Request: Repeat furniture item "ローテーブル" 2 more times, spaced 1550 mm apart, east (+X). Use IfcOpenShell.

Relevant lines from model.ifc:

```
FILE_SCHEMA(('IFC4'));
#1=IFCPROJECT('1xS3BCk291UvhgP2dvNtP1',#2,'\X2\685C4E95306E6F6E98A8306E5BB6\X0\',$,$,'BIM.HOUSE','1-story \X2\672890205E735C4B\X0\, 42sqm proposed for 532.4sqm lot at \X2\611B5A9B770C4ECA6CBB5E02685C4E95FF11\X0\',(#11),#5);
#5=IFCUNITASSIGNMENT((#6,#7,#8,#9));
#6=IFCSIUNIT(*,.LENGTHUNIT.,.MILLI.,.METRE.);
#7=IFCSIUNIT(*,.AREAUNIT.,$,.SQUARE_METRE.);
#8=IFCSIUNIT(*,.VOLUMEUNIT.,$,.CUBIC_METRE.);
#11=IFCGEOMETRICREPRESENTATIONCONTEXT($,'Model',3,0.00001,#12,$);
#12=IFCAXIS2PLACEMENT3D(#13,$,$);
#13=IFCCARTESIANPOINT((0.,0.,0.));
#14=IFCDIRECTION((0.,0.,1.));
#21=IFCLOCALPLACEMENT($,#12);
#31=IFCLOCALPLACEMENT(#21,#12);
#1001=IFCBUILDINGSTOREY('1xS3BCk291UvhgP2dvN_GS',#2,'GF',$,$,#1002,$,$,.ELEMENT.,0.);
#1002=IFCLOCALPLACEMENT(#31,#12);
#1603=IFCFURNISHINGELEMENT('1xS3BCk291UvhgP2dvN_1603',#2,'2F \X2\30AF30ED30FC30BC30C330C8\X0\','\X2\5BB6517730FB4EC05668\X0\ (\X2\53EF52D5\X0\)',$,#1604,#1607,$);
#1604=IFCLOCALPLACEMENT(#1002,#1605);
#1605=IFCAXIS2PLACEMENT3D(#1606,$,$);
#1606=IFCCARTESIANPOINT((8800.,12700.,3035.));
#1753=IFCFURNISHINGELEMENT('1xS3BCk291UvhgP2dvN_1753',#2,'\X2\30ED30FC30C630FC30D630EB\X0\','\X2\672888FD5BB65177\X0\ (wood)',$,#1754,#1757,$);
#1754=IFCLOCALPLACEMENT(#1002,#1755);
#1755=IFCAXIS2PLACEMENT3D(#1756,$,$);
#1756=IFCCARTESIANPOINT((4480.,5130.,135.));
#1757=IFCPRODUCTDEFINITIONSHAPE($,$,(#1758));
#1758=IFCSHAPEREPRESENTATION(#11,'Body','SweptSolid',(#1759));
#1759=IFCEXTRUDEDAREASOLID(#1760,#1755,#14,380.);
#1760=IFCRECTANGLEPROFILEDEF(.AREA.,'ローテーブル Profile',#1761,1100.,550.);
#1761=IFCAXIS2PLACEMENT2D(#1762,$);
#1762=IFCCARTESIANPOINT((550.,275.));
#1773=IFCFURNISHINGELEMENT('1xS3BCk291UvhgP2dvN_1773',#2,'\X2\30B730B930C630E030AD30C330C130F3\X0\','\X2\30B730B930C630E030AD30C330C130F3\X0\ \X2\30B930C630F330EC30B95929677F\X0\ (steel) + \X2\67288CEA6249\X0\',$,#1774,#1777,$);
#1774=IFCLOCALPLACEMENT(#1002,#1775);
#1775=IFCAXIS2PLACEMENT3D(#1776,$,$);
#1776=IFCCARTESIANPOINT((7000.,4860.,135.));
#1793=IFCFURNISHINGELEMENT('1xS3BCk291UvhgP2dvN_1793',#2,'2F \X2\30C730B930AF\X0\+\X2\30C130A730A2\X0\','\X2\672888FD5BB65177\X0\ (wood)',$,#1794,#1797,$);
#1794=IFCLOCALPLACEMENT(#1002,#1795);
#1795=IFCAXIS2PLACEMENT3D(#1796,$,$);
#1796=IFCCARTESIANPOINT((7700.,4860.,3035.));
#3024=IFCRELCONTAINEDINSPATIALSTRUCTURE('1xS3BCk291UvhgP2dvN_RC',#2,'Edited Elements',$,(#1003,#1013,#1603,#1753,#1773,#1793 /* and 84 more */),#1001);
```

```python
import numpy as np
import ifcopenshell
import ifcopenshell.api.geometry
import ifcopenshell.api.root
import ifcopenshell.util.element
import ifcopenshell.util.placement

model = ifcopenshell.open("model.ifc")


def reuse_history(source, copy):
    """copy_class also copies each property set's owner history, people and application; keep the originals."""
    for rel in copy.IsDefinedBy:
        if rel.is_a("IfcRelDefinesByProperties") and (history := rel.RelatingPropertyDefinition.OwnerHistory):
            rel.RelatingPropertyDefinition.OwnerHistory = source.OwnerHistory
            ifcopenshell.util.element.remove_deep2(model, history)


source = model.by_guid("1xS3BCk291UvhgP2dvN_1753")
base = ifcopenshell.util.placement.get_local_placement(source.ObjectPlacement)
step = np.array([1.0, 0.0, 0.0]) * 1550.0

for i in range(1, 3):
    copy = ifcopenshell.api.root.copy_class(model, product=source)
    copy.Representation = ifcopenshell.util.element.copy_deep(
        model, source.Representation, exclude=["IfcGeometricRepresentationContext", "IfcRepresentationMap"]
    )
    reuse_history(source, copy)
    matrix = base.copy()
    matrix[:3, 3] += i * step
    print("added at", matrix[:3, 3].round(3) + 0.0)
    ifcopenshell.api.geometry.edit_object_placement(model, product=copy, matrix=matrix, is_si=False)

model.write("model_rev.ifc")
```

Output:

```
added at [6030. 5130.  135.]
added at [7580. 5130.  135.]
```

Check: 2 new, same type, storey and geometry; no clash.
